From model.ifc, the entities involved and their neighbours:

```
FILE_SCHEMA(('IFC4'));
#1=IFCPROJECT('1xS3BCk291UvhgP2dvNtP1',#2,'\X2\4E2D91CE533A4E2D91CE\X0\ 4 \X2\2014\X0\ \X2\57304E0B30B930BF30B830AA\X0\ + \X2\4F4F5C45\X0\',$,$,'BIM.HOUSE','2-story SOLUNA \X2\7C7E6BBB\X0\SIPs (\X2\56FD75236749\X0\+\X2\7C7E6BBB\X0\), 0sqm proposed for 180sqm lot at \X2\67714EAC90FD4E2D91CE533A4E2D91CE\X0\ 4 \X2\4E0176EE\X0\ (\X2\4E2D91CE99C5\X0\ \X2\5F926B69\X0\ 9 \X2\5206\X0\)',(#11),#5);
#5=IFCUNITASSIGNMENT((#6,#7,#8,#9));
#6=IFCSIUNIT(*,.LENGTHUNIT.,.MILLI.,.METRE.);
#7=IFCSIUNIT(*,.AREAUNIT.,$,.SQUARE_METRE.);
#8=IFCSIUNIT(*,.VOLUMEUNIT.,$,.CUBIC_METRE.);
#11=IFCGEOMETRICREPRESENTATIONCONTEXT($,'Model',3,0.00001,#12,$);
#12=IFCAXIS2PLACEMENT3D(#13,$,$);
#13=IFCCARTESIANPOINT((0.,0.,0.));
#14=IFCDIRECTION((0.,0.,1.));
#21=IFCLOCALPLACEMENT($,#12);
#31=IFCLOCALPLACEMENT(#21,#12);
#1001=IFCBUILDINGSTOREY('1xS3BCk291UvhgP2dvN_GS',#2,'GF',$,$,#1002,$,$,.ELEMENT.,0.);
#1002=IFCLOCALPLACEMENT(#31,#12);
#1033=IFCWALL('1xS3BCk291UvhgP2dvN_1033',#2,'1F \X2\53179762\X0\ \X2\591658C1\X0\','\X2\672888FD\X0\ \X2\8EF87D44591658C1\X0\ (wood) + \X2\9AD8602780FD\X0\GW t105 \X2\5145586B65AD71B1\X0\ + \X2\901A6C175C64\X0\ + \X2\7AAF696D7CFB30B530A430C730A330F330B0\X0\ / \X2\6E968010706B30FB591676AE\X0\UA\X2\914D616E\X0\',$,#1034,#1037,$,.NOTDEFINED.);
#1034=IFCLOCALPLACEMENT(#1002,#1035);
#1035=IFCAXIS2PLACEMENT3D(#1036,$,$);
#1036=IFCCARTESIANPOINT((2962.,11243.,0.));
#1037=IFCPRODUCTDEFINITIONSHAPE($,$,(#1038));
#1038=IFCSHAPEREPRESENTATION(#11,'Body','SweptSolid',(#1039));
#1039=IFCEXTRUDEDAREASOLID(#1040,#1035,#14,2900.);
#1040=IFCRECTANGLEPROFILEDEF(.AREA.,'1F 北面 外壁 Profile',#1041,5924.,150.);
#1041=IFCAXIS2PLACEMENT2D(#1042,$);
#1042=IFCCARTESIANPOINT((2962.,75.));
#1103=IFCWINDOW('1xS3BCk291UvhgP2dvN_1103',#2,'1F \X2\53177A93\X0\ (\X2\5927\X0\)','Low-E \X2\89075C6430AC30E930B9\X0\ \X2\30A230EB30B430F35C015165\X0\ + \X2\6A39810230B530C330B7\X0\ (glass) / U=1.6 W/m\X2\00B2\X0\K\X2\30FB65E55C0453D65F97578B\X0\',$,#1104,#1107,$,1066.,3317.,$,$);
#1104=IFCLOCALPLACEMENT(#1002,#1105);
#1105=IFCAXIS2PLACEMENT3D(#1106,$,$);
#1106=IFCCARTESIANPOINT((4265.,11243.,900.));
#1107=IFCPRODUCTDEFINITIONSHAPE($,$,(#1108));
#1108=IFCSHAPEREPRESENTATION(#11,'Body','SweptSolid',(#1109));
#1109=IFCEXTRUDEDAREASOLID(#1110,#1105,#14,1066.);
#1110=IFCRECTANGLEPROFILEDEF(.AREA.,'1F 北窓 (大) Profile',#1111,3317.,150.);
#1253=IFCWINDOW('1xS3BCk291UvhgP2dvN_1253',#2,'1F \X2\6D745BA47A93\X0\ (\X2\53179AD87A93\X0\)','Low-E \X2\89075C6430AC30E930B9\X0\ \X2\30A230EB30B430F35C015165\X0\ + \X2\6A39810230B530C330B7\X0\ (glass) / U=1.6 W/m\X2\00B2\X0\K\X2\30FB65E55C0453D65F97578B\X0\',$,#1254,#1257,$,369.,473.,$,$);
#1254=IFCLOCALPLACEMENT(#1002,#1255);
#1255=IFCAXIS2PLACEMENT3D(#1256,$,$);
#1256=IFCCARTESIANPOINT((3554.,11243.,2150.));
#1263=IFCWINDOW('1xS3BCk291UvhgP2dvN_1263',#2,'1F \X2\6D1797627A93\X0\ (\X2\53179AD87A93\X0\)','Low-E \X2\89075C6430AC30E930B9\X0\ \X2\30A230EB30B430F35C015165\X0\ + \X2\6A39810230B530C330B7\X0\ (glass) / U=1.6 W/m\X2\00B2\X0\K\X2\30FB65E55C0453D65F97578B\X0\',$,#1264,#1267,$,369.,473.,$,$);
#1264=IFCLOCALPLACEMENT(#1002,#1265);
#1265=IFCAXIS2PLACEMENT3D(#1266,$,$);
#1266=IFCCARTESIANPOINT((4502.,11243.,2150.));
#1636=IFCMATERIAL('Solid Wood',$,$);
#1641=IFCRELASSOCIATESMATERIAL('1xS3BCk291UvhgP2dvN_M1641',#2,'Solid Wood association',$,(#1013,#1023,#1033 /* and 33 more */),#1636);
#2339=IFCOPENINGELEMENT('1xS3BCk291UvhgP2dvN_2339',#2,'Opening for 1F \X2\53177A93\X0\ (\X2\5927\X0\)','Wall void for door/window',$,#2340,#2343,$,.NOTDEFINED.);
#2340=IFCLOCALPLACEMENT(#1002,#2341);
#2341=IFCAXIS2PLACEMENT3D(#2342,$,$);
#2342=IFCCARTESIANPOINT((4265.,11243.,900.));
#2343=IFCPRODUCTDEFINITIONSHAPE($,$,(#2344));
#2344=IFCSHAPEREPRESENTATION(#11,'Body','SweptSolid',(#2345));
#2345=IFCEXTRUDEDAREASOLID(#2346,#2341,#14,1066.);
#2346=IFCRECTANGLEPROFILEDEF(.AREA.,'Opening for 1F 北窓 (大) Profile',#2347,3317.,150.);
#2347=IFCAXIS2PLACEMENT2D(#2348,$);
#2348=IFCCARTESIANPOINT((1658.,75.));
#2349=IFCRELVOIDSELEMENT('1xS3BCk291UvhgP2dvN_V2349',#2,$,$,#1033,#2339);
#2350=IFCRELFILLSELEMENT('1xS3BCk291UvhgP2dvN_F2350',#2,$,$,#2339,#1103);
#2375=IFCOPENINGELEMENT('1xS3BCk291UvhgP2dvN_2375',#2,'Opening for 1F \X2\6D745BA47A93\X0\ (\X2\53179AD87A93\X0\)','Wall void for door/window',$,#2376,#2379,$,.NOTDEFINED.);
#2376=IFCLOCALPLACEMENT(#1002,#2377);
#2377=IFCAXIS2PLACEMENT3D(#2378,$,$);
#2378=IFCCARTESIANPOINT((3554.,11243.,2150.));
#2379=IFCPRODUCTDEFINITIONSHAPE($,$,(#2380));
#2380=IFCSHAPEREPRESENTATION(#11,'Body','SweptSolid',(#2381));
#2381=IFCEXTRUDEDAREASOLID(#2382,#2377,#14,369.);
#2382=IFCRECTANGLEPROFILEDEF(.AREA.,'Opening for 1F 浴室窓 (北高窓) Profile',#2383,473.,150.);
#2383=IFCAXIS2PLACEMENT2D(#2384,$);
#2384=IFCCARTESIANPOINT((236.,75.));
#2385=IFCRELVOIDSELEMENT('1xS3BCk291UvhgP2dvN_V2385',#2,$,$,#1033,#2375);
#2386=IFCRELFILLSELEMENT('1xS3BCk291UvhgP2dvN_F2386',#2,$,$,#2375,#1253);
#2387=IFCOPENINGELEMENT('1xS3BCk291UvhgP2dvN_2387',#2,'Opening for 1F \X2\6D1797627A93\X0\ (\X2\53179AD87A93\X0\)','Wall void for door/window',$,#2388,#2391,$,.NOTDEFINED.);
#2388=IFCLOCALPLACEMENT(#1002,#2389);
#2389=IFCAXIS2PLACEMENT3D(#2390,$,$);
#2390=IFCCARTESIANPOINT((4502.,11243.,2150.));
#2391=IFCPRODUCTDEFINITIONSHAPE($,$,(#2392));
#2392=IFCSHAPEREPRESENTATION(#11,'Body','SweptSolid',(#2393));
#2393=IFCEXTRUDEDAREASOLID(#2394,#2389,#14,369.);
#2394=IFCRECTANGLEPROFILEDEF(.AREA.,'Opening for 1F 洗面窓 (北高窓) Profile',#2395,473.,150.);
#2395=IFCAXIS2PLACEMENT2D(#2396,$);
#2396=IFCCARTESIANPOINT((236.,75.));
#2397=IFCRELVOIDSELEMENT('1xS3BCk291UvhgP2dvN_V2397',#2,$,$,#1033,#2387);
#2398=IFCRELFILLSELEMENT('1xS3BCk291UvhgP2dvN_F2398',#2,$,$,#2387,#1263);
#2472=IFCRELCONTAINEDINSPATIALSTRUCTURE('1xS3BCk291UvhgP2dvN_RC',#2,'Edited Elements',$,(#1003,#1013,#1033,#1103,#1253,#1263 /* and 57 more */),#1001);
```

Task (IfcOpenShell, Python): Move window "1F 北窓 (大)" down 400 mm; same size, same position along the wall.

```python
import numpy as np
import ifcopenshell
import ifcopenshell.api.geometry
import ifcopenshell.util.placement
import ifcopenshell.util.unit

model = ifcopenshell.open("model.ifc")
unit_scale = ifcopenshell.util.unit.calculate_unit_scale(model)

window = model.by_guid("1xS3BCk291UvhgP2dvN_1103")
opening = window.FillsVoids[0].RelatingOpeningElement
dz = -400.0

shift = np.array([0.0, 0.0, dz])
# The window is not placed relative to its opening, so move both.
for product in (opening, window):
    matrix = ifcopenshell.util.placement.get_local_placement(product.ObjectPlacement)
    matrix[:3, 3] += shift
    ifcopenshell.api.geometry.edit_object_placement(model, product=product, matrix=matrix, is_si=False)

print(f"moved by {dz * unit_scale:+.3f} m")

model.write("model_v2.ifc")
```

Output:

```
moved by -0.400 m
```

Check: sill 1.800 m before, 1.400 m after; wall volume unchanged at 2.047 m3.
